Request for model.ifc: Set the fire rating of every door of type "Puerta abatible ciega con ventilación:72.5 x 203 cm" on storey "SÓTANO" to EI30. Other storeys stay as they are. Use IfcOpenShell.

First a look at what the model holds.

```python
import ifcopenshell
import ifcopenshell.util.element

model = ifcopenshell.open("model.ifc")
print(model.schema)
storey = next(s for s in model.by_type("IfcBuildingStorey") if s.Name == "SÓTANO")
doors = [e for e in ifcopenshell.util.element.get_decomposition(storey) if e.is_a("IfcDoor")]
seen = {}
for e in doors:
    element_type = ifcopenshell.util.element.get_type(e)
    key = (element_type.Name if element_type != e and element_type else None, ifcopenshell.util.element.get_pset(e, "Pset_DoorCommon", "FireRating"))
    seen[key] = seen.get(key, 0) + 1
for (name, value), count in sorted(seen.items(), key=str):
    print(count, "x", name, "|", value)
```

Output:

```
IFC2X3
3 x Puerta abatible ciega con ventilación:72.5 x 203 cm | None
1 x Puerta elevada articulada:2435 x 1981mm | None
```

```python
import ifcopenshell
import ifcopenshell.api.pset
import ifcopenshell.util.element

model = ifcopenshell.open("model.ifc")

storey = next(s for s in model.by_type("IfcBuildingStorey") if s.Name == "SÓTANO")
doors = [e for e in ifcopenshell.util.element.get_decomposition(storey) if e.is_a("IfcDoor")]

count = 0
for e in doors:
    element_type = ifcopenshell.util.element.get_type(e)
    if element_type in (None, e) or element_type.Name != "Puerta abatible ciega con ventilación:72.5 x 203 cm":
        continue
    # add_pset returns the element's existing set when there is one.
    pset = ifcopenshell.api.pset.add_pset(model, product=e, name="Pset_DoorCommon")
    ifcopenshell.api.pset.edit_pset(model, pset=pset, properties={"FireRating": "EI30"})
    count += 1

print(count, "doors updated")

model.write("model_updated.ifc")
```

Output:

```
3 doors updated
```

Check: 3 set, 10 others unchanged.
